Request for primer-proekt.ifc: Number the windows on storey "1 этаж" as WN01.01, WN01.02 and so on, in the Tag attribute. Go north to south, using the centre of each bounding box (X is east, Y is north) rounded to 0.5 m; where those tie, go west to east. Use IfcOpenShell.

First a look at what the model holds.

```python
import ifcopenshell
import ifcopenshell.util.element
import ifcopenshell.util.placement

model = ifcopenshell.open("primer-proekt.ifc")
print(model.schema)
storey = next(s for s in model.by_type("IfcBuildingStorey") if s.Name == "1 этаж")
windows = [e for e in ifcopenshell.util.element.get_decomposition(storey) if e.is_a("IfcWindow")]
for e in sorted(windows, key=lambda e: e.id()):
    origin = ifcopenshell.util.placement.get_local_placement(e.ObjectPlacement)[:3, 3]
    print(e.id(), e.Tag, e.Name, origin.round(2) + 0.0, sep=" | ")
```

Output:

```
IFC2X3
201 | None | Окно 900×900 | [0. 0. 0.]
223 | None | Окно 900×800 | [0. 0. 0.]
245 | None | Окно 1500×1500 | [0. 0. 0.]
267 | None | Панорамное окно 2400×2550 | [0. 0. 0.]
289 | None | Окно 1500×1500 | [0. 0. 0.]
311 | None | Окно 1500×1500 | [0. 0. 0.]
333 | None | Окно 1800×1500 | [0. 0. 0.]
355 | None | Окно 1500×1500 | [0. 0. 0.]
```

```python
import ifcopenshell
import ifcopenshell.geom
import ifcopenshell.util.element
import ifcopenshell.util.shape

model = ifcopenshell.open("primer-proekt.ifc")
settings = ifcopenshell.geom.settings()
settings.set("use-world-coords", True)


def centre(element):
    shape = ifcopenshell.geom.create_shape(settings, element)
    return ifcopenshell.util.shape.get_bbox_centroid(shape.geometry)


storey = next(s for s in model.by_type("IfcBuildingStorey") if s.Name == "1 этаж")
windows = [e for e in ifcopenshell.util.element.get_decomposition(storey) if e.is_a("IfcWindow")]

# Insertion points can sit at a corner or the storey origin, so sort by the geometry (in metres).
centres = {e: centre(e) for e in windows}
windows.sort(key=lambda e: (-round(centres[e][1] / 0.5), centres[e][0]))

for i, e in enumerate(windows, start=1):
    number = f"WN01.{i:02d}"
    e.Tag = number
    print(e.id(), number)

model.write("primer-proekt_edited.ifc")
```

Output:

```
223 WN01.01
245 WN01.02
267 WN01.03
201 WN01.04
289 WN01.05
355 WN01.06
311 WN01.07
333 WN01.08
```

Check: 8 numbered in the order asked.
